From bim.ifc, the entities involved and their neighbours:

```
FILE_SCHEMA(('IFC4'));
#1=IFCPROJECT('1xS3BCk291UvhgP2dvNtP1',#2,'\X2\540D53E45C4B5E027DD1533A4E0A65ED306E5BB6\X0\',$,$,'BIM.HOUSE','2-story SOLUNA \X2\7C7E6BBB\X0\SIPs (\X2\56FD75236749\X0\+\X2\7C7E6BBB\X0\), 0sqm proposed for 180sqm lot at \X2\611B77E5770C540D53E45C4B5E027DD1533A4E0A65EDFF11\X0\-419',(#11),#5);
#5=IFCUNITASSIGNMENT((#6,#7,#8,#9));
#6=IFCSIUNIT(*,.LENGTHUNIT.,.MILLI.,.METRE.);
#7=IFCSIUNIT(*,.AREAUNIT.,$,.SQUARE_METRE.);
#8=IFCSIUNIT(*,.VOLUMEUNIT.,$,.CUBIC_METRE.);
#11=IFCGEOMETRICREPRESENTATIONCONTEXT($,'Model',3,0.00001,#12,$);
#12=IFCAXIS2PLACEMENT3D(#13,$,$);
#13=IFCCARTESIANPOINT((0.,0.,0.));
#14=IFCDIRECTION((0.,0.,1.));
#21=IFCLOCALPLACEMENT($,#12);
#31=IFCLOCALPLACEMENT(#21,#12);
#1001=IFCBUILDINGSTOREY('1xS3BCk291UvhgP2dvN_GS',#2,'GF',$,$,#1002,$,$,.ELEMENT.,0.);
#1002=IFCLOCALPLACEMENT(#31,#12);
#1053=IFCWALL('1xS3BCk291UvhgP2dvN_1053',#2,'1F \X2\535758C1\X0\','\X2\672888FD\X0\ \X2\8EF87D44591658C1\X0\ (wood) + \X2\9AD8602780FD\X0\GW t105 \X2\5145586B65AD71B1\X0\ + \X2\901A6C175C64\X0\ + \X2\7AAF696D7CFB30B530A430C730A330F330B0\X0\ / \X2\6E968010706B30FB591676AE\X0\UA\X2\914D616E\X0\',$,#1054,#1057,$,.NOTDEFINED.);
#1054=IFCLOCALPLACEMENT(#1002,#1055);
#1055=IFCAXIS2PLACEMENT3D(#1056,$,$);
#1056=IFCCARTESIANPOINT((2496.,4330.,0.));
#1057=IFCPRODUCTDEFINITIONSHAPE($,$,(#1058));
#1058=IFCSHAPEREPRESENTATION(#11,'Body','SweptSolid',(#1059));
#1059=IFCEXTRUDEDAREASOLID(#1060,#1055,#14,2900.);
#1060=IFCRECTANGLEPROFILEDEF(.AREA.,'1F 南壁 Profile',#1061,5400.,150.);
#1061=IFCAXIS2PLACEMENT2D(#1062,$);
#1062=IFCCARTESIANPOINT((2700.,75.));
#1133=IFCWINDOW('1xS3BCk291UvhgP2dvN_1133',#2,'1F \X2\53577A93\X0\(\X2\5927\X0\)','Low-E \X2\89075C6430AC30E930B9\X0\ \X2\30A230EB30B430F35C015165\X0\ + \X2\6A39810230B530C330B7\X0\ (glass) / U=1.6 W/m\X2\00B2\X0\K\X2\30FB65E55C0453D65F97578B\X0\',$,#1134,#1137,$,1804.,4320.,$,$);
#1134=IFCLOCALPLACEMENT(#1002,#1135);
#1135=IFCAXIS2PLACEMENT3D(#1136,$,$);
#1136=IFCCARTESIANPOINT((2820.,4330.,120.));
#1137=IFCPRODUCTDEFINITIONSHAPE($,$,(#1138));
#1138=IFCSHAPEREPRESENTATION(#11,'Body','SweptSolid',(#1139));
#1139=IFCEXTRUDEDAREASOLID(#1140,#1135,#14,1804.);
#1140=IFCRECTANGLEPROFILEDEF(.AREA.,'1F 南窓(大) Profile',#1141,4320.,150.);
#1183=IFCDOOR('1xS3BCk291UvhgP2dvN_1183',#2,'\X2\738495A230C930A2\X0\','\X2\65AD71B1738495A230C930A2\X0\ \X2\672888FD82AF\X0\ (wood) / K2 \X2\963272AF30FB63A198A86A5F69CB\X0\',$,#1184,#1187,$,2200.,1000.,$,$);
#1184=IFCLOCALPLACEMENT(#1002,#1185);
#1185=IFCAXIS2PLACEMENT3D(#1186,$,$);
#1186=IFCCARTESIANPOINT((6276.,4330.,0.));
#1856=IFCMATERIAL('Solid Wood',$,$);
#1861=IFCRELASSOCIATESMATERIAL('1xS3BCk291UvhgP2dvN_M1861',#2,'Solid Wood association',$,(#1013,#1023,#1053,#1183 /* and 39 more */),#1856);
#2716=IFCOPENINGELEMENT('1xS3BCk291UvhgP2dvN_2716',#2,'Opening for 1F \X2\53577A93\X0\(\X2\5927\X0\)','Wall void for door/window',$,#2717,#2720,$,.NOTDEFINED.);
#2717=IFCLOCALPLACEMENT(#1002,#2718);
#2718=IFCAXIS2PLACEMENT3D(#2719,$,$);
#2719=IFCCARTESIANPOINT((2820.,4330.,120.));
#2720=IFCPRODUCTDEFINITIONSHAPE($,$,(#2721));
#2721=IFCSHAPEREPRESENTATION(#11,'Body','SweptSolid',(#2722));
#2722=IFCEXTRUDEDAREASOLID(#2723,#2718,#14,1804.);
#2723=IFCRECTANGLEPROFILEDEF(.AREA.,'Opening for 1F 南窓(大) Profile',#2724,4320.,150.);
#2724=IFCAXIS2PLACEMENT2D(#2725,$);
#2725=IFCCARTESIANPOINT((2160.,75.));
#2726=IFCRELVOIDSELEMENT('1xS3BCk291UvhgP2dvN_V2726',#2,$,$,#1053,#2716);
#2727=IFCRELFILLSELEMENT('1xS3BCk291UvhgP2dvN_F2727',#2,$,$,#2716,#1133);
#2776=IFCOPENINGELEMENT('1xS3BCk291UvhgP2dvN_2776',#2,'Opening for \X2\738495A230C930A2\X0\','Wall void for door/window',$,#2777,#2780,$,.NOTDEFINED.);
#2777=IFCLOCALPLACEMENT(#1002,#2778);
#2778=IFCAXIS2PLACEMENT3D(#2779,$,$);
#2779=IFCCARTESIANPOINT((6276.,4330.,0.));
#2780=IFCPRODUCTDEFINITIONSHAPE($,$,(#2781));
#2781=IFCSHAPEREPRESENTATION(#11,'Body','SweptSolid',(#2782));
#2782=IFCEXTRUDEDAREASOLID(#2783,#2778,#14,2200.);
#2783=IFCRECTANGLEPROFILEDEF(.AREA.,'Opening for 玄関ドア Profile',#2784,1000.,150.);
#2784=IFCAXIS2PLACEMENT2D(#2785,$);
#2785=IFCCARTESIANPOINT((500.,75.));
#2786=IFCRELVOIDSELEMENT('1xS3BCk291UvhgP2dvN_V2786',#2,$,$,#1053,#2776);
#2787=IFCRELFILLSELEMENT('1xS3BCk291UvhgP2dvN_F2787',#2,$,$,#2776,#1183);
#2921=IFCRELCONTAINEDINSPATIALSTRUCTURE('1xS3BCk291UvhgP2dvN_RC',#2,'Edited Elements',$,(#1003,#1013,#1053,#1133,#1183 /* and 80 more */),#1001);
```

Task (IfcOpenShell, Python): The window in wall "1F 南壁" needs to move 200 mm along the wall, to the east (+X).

```python
import ifcopenshell
import ifcopenshell.api.geometry
import ifcopenshell.util.placement
import ifcopenshell.util.unit

model = ifcopenshell.open("bim.ifc")
unit_scale = ifcopenshell.util.unit.calculate_unit_scale(model)

window = model.by_guid("1xS3BCk291UvhgP2dvN_1133")
opening = window.FillsVoids[0].RelatingOpeningElement
wall = opening.VoidsElements[0].RelatingBuildingElement

wall_matrix = ifcopenshell.util.placement.get_local_placement(wall.ObjectPlacement)
shift = wall_matrix[:3, 0] * 0.2 / unit_scale
before = ifcopenshell.util.placement.get_local_placement(window.ObjectPlacement)[:3, 3].copy()

# The window is not placed relative to its opening, so move both.
for product in (opening, window):
    matrix = ifcopenshell.util.placement.get_local_placement(product.ObjectPlacement)
    matrix[:3, 3] += shift
    ifcopenshell.api.geometry.edit_object_placement(model, product=product, matrix=matrix, is_si=False)

after = ifcopenshell.util.placement.get_local_placement(window.ObjectPlacement)[:3, 3]
print("window moved by", (after - before).round(3) + 0.0)

model.write("bim-out.ifc")
```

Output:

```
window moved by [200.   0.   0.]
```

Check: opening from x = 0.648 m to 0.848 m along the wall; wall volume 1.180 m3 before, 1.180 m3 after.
